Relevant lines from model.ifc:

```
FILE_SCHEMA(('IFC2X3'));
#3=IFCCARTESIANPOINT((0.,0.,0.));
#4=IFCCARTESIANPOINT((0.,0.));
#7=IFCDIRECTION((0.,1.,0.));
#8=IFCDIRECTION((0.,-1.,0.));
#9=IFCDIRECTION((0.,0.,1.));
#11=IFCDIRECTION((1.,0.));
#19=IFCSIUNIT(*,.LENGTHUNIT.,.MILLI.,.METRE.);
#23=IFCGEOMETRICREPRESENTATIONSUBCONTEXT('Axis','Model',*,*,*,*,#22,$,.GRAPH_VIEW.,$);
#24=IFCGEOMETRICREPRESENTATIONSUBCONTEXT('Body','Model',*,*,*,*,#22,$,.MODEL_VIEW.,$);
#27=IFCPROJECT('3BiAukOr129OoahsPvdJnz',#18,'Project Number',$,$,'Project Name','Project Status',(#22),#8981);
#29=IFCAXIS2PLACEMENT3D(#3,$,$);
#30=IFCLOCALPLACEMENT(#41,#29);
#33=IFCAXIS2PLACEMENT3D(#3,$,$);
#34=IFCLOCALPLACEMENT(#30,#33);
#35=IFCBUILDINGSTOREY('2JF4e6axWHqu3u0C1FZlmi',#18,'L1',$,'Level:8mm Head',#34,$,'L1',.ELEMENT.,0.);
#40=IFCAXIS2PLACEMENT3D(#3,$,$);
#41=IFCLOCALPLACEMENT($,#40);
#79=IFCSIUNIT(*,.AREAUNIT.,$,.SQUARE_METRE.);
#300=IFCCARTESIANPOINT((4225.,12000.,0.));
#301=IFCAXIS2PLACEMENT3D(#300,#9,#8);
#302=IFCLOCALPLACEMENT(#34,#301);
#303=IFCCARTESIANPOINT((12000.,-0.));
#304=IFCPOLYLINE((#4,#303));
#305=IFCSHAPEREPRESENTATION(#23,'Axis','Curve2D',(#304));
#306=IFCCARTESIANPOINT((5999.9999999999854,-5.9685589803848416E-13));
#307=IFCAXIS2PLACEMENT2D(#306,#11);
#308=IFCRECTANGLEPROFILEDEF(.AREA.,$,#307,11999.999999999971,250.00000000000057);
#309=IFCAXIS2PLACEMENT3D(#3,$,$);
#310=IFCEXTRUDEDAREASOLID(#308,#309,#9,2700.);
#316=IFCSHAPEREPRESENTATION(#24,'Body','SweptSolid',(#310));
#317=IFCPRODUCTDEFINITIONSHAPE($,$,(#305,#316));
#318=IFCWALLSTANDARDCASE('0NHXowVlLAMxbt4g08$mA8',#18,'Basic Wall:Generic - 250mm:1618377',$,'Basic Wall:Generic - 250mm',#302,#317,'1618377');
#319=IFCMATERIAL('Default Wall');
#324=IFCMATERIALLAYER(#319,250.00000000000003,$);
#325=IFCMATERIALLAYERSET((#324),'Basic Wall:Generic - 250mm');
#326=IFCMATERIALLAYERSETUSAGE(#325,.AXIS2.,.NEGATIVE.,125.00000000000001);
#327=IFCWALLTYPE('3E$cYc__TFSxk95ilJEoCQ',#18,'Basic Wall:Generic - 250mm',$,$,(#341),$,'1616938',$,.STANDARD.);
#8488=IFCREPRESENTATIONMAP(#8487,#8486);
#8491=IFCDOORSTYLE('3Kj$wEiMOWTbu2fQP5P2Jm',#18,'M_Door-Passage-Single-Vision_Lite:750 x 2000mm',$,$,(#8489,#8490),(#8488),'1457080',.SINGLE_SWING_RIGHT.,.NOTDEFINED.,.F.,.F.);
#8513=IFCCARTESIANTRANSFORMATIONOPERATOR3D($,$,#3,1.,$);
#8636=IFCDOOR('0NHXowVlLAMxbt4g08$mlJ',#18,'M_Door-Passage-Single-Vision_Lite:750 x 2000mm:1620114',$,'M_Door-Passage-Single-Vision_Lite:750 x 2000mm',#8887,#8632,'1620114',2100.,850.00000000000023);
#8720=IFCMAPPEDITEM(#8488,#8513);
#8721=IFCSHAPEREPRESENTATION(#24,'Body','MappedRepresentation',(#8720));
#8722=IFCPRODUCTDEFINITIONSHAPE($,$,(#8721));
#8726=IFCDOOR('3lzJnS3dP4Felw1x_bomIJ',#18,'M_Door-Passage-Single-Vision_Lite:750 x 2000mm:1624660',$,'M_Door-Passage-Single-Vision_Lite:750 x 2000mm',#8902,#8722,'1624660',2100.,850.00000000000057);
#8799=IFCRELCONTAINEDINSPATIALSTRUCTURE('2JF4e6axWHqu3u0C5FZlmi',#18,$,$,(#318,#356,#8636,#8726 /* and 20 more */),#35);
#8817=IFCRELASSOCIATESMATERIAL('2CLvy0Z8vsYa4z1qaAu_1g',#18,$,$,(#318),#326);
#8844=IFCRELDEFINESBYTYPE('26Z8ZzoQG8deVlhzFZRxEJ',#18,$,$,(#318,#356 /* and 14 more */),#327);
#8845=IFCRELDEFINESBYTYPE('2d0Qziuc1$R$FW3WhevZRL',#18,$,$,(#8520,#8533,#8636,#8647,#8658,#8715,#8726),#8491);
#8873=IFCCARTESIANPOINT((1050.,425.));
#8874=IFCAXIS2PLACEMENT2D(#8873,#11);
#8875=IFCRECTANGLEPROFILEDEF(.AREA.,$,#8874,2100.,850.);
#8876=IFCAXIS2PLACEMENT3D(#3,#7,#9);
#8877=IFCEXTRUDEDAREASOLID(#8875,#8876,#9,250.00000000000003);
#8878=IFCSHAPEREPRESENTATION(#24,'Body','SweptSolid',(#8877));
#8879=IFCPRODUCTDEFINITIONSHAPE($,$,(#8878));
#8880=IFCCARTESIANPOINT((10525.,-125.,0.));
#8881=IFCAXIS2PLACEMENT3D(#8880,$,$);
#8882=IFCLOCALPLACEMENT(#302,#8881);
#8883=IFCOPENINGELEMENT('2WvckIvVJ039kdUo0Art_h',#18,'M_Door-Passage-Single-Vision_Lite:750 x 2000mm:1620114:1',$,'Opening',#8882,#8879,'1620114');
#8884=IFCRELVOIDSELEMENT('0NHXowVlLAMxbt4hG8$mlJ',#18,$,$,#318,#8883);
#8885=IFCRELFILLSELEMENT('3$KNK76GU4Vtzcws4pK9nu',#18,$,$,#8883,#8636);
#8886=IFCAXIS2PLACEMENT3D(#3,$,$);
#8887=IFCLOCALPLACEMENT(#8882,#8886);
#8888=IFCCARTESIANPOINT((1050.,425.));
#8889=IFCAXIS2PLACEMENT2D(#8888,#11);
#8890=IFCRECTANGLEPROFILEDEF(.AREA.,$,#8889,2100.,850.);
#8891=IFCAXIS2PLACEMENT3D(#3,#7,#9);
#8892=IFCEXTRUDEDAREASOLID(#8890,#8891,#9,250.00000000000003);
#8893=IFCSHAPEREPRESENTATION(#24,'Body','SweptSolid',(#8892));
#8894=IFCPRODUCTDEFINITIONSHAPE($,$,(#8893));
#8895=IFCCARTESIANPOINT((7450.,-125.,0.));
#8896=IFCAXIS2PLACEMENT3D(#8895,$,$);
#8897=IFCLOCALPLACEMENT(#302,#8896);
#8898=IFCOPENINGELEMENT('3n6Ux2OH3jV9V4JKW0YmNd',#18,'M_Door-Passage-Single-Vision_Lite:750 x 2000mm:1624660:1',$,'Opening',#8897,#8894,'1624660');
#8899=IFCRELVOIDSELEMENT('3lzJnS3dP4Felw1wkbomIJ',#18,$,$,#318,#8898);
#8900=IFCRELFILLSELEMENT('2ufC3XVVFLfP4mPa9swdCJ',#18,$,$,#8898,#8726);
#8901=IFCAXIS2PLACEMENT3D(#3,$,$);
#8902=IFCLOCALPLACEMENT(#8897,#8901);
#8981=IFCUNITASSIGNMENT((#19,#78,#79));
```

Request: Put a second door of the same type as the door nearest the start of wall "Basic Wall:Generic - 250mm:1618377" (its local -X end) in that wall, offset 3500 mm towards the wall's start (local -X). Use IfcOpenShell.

```python
import ifcopenshell
import ifcopenshell.api.feature
import ifcopenshell.api.geometry
import ifcopenshell.api.root
import ifcopenshell.geom
import ifcopenshell.util.element
import ifcopenshell.util.placement
import ifcopenshell.util.shape
import ifcopenshell.util.unit

model = ifcopenshell.open("model.ifc")
unit_scale = ifcopenshell.util.unit.calculate_unit_scale(model)
settings = ifcopenshell.geom.settings()


def volume(element):
    """Net volume in cubic metres, openings subtracted."""
    shape = ifcopenshell.geom.create_shape(settings, element)
    return ifcopenshell.util.shape.get_volume(shape.geometry)


def reuse_history(source, copy):
    """copy_class also copies each property set's owner history, people and application; keep the originals."""
    for rel in copy.IsDefinedBy:
        if rel.is_a("IfcRelDefinesByProperties") and (history := rel.RelatingPropertyDefinition.OwnerHistory):
            rel.RelatingPropertyDefinition.OwnerHistory = source.OwnerHistory
            ifcopenshell.util.element.remove_deep2(model, history)


door = model.by_guid("3lzJnS3dP4Felw1x_bomIJ")
opening = door.FillsVoids[0].RelatingOpeningElement
wall = opening.VoidsElements[0].RelatingBuildingElement
before = volume(wall)
shift = ifcopenshell.util.placement.get_local_placement(wall.ObjectPlacement)[:3, 0] * -3.5 / unit_scale

# copy_class copies the void relationship, type, container and properties, but no geometry.
new_opening = ifcopenshell.api.root.copy_class(model, product=opening)
new_opening.Representation = ifcopenshell.util.element.copy_deep(
    model, opening.Representation, exclude=["IfcGeometricRepresentationContext", "IfcRepresentationMap"]
)
new_opening.Name = "M_Door-Passage-Single-Vision_Lite:750 x 2000mm"
new_opening.Tag = None
new_door = ifcopenshell.api.root.copy_class(model, product=door)
new_door.Representation = ifcopenshell.util.element.copy_deep(
    model, door.Representation, exclude=["IfcGeometricRepresentationContext", "IfcRepresentationMap"]
)
new_door.Name = "M_Door-Passage-Single-Vision_Lite:750 x 2000mm"
new_door.Tag = None
reuse_history(door, new_door)
fills = ifcopenshell.api.feature.add_filling(model, opening=new_opening, element=new_door)
fills.OwnerHistory = new_door.OwnerHistory  # required in IFC2X3

for old, new in ((opening, new_opening), (door, new_door)):
    matrix = ifcopenshell.util.placement.get_local_placement(old.ObjectPlacement)
    matrix[:3, 3] += shift
    ifcopenshell.api.geometry.edit_object_placement(model, product=new, matrix=matrix, is_si=False)

after = volume(wall)

print(f"wall volume {before:.3f} -> {after:.3f} m3")

model.write("model_updated.ifc")
```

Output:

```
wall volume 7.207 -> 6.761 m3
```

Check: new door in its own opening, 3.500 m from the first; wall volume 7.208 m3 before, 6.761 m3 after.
